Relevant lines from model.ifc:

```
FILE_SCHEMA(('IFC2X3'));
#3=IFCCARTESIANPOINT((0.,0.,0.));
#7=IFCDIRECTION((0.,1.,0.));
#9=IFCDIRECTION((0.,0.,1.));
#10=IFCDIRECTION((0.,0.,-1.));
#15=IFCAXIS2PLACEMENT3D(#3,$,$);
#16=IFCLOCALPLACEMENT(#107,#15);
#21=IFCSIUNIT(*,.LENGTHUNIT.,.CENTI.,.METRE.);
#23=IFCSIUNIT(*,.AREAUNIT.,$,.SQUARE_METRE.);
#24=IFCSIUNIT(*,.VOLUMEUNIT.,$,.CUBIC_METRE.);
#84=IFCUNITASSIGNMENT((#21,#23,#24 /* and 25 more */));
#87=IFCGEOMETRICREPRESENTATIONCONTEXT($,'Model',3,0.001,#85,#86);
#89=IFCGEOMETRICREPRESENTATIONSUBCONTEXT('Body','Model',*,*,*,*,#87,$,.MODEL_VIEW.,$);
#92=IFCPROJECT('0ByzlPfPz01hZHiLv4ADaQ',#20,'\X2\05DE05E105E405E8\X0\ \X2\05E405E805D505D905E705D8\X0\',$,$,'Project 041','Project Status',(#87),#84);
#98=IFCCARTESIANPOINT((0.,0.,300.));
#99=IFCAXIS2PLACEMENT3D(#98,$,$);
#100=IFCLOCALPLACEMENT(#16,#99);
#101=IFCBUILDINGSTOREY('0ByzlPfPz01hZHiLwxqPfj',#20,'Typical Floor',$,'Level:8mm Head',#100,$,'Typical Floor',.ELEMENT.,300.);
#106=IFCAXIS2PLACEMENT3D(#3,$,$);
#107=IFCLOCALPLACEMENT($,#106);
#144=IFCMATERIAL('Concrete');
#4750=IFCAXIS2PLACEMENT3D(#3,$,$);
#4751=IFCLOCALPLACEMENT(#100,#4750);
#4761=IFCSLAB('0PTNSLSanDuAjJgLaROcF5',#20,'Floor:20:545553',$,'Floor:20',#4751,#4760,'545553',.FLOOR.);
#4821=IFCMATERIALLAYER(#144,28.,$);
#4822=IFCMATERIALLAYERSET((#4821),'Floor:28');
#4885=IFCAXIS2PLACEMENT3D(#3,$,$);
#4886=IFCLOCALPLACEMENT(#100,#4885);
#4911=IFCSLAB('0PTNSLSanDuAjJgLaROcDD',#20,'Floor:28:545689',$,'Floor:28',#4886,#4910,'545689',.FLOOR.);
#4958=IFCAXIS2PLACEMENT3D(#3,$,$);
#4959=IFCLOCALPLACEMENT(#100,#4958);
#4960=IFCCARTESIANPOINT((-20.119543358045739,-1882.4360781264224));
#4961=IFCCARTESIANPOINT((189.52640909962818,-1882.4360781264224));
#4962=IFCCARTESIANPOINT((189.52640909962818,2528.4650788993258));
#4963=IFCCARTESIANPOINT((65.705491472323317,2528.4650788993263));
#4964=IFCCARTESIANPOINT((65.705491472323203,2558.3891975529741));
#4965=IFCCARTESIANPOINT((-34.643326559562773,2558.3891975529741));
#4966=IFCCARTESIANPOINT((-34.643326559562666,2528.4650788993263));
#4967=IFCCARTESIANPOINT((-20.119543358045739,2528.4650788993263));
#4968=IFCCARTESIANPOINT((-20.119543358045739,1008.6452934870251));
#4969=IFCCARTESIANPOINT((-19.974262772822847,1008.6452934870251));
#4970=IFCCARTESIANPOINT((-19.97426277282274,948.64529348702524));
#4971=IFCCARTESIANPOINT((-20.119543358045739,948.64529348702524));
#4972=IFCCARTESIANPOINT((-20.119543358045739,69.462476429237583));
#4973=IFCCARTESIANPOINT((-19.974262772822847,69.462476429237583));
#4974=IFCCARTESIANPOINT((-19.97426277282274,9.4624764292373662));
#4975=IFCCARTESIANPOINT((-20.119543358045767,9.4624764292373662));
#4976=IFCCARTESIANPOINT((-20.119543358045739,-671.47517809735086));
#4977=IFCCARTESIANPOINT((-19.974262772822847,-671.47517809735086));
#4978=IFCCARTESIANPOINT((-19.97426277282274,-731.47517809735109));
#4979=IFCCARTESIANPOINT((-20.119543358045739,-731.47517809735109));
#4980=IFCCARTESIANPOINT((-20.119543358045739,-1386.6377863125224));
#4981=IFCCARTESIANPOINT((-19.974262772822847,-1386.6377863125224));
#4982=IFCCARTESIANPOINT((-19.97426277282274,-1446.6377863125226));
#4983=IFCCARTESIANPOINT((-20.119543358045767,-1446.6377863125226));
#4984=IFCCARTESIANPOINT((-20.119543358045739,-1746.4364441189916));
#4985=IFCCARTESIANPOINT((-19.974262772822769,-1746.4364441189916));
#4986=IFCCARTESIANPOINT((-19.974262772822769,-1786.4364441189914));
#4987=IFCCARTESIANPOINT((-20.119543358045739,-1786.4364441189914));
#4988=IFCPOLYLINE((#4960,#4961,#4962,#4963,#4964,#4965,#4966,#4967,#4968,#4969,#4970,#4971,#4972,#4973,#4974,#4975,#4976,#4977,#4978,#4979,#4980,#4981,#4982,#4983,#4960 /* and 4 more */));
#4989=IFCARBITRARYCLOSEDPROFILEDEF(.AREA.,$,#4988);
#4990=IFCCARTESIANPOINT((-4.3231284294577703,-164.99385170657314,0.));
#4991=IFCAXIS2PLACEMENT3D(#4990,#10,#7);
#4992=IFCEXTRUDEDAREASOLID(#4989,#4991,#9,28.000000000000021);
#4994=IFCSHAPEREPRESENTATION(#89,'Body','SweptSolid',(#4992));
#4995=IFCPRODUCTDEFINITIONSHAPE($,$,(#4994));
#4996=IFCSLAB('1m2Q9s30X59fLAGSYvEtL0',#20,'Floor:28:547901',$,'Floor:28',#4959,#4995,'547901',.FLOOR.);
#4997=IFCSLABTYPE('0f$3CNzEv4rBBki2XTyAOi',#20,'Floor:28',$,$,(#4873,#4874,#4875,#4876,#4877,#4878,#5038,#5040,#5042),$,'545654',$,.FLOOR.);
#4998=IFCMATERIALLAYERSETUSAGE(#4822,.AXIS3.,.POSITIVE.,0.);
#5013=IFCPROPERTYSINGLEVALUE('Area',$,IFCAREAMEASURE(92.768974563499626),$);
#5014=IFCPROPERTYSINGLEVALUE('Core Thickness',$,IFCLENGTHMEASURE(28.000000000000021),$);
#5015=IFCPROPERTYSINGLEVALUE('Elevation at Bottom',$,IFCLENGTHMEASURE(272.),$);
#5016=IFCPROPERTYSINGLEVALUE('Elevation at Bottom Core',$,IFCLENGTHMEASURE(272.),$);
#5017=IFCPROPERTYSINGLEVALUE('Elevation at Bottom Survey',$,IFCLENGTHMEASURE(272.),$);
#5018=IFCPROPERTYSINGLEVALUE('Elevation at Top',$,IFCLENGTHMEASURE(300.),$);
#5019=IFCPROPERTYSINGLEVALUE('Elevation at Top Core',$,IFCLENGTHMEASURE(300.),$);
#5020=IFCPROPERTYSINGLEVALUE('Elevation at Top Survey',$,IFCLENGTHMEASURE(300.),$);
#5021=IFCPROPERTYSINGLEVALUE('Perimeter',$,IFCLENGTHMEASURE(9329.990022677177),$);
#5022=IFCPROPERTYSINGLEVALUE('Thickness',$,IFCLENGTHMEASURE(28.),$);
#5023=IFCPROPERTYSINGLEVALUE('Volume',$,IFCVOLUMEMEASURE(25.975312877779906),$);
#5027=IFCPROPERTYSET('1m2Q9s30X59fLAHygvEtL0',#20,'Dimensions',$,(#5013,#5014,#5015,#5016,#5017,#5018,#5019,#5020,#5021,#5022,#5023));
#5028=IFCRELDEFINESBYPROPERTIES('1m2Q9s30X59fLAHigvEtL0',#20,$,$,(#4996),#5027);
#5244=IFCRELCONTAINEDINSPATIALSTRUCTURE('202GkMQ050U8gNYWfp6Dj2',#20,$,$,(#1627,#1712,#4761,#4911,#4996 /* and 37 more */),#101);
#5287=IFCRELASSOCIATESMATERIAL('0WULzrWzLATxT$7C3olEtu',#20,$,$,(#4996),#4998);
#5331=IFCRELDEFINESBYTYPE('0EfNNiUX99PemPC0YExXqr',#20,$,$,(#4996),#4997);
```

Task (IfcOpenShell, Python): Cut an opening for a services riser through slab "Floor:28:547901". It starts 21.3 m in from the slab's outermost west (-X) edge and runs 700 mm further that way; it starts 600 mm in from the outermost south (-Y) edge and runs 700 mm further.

```python
import numpy as np
import ifcopenshell
import ifcopenshell.api.feature
import ifcopenshell.api.geometry
import ifcopenshell.api.pset
import ifcopenshell.api.root
import ifcopenshell.geom
import ifcopenshell.util.element
import ifcopenshell.util.placement
import ifcopenshell.util.representation
import ifcopenshell.util.shape
import ifcopenshell.util.unit

model = ifcopenshell.open("model.ifc")
unit_scale = ifcopenshell.util.unit.calculate_unit_scale(model)
area_scale = ifcopenshell.util.unit.calculate_unit_scale(model, "AREAUNIT")
volume_scale = ifcopenshell.util.unit.calculate_unit_scale(model, "VOLUMEUNIT")
settings = ifcopenshell.geom.settings()


def volume(element):
    """Net volume in cubic metres, openings subtracted."""
    shape = ifcopenshell.geom.create_shape(settings, element)
    return ifcopenshell.util.shape.get_volume(shape.geometry)


slab = model.by_id(4996)
before = volume(slab)

# Extent in the slab's own axes, in metres. The edges named are its -X and -Y sides.
slab_shape = ifcopenshell.geom.create_shape(settings, slab)
vertices = ifcopenshell.util.shape.get_vertices(slab_shape.geometry)
x_min, y_min, bottom = vertices.min(axis=0)
top = vertices[:, 2].max()

opening = ifcopenshell.api.root.create_entity(model, ifc_class="IfcOpeningElement", name="Services riser opening")
context = ifcopenshell.util.representation.get_context(model, "Model", "Body", "MODEL_VIEW")
width, depth = 0.7, 0.7
outline = [(0.0, 0.0), (width, 0.0), (width, depth), (0.0, depth), (0.0, 0.0)]
# Overshoot both faces by 50 mm so the cut is clean.
shape = ifcopenshell.api.geometry.add_slab_representation(
    model, context=context, depth=top - bottom + 0.1, polyline=outline
)
ifcopenshell.api.geometry.assign_representation(model, product=opening, representation=shape)

matrix = ifcopenshell.util.placement.get_local_placement(slab.ObjectPlacement)
matrix[:, 3] = matrix @ np.append(np.array([x_min + 21.3, y_min + 0.6, bottom - 0.05]) / unit_scale, 1.0)
ifcopenshell.api.geometry.edit_object_placement(model, product=opening, matrix=matrix, is_si=False)
ifcopenshell.api.feature.add_feature(model, feature=opening, element=slab)

after = volume(slab)

# Update the slab's stored quantities.
pset = model.by_id(ifcopenshell.util.element.get_pset(slab, "Dimensions", should_inherit=False)["id"])
ifcopenshell.api.pset.edit_pset(model, pset=pset, properties={
    "Area": model.create_entity("IfcAreaMeasure", after / (top - bottom) / area_scale),
    "Volume": model.create_entity("IfcVolumeMeasure", after / volume_scale),
})

print(f"slab volume {before:.3f} -> {after:.3f} m3")

model.write("model_updated.ifc")
```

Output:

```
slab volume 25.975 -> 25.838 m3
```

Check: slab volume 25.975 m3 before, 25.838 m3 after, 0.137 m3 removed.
